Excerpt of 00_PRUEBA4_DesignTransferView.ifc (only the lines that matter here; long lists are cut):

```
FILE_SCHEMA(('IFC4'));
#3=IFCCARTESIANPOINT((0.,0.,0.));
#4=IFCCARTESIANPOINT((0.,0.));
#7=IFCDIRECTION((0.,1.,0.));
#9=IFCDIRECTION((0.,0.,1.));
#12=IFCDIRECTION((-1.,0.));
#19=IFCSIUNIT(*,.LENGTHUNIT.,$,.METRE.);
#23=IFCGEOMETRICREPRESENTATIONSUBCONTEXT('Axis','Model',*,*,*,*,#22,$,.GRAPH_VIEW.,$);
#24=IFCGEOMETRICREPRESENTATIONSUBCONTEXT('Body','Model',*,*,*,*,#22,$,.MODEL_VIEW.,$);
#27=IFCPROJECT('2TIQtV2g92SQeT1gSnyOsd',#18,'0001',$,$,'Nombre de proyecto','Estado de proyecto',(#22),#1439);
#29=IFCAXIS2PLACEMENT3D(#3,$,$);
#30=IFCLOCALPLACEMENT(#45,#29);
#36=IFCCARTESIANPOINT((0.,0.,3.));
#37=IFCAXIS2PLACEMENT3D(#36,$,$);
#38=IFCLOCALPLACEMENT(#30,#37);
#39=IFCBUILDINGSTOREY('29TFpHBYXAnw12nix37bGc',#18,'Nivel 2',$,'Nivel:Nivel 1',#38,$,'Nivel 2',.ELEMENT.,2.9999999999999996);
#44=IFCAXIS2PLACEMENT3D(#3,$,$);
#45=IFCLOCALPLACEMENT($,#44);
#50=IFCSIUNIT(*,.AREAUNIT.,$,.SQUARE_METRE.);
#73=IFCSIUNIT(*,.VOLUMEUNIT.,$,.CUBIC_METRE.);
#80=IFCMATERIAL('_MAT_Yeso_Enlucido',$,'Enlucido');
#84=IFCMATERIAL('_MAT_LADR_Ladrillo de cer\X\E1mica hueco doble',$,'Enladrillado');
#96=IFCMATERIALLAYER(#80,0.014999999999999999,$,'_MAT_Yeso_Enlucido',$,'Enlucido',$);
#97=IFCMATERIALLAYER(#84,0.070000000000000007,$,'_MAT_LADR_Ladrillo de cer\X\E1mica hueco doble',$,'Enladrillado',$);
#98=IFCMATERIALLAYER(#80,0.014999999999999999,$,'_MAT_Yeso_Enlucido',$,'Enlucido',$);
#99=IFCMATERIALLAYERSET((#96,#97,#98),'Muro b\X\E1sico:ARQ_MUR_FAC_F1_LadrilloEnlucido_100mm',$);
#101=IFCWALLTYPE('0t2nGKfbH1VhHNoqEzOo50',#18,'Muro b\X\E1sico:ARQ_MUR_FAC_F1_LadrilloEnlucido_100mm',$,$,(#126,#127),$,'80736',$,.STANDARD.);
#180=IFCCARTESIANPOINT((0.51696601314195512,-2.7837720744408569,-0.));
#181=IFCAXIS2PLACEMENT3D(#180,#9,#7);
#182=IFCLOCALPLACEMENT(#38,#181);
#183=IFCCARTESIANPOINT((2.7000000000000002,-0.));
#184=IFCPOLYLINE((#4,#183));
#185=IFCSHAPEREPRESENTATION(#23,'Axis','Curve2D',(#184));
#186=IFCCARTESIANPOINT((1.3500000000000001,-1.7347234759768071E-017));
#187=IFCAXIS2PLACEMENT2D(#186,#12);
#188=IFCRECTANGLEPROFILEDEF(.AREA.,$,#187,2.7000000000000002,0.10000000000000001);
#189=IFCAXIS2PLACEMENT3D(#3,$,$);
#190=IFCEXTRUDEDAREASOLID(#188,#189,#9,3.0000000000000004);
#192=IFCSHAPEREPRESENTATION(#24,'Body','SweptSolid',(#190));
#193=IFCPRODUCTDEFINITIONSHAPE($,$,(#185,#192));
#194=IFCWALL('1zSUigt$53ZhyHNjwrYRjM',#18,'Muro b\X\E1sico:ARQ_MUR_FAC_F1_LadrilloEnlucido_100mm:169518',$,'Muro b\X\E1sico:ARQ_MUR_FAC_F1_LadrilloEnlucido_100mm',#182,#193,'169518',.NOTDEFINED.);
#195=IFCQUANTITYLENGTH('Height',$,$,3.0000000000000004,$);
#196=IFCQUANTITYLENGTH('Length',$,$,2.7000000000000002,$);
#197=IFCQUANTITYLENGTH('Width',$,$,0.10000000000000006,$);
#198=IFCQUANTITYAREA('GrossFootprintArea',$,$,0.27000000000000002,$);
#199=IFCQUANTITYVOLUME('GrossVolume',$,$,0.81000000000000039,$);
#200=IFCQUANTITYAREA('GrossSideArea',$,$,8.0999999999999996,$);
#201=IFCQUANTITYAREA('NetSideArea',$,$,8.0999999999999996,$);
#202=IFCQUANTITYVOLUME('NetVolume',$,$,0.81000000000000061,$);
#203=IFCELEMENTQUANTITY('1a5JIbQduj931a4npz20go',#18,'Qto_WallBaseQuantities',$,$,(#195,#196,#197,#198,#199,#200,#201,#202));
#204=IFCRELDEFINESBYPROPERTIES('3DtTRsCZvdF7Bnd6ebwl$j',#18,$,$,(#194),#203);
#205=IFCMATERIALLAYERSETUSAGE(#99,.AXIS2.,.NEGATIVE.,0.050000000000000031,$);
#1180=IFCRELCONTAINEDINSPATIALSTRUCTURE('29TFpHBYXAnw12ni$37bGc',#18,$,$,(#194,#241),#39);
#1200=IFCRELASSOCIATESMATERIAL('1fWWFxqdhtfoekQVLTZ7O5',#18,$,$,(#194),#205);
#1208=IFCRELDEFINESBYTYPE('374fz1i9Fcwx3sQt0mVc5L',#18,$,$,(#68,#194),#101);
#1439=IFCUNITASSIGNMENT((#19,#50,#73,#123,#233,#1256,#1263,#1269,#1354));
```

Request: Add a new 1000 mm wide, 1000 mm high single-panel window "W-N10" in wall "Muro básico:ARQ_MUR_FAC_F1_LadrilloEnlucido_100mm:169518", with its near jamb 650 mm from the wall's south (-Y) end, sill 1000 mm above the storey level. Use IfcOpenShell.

```python
import numpy as np
import ifcopenshell
import ifcopenshell.api.feature
import ifcopenshell.api.geometry
import ifcopenshell.api.pset
import ifcopenshell.api.root
import ifcopenshell.api.spatial
import ifcopenshell.geom
import ifcopenshell.util.element
import ifcopenshell.util.placement
import ifcopenshell.util.representation
import ifcopenshell.util.shape
import ifcopenshell.util.unit

model = ifcopenshell.open("00_PRUEBA4_DesignTransferView.ifc")
unit_scale = ifcopenshell.util.unit.calculate_unit_scale(model)
area_scale = ifcopenshell.util.unit.calculate_unit_scale(model, "AREAUNIT")
volume_scale = ifcopenshell.util.unit.calculate_unit_scale(model, "VOLUMEUNIT")
settings = ifcopenshell.geom.settings()


def volume(element):
    """Net volume in cubic metres, openings subtracted."""
    shape = ifcopenshell.geom.create_shape(settings, element)
    return ifcopenshell.util.shape.get_volume(shape.geometry)


wall = model.by_guid("1zSUigt$53ZhyHNjwrYRjM")
storey = ifcopenshell.util.element.get_container(wall, ifc_class="IfcBuildingStorey")
context = ifcopenshell.util.representation.get_context(model, "Model", "Body", "MODEL_VIEW")
before = volume(wall)

width, height, from_end, sill = 1, 1, 0.65, 1  # metres

# The wall runs along its own X axis, and the end named is its -X end.
wall_shape = ifcopenshell.geom.create_shape(settings, wall)
x, y, z = ifcopenshell.util.shape.get_vertices(wall_shape.geometry).T
start = x.min() + from_end
face, thickness = float(y.min()), float(y.max() - y.min())
wall_matrix = ifcopenshell.util.placement.get_local_placement(wall.ObjectPlacement)
level = ifcopenshell.util.placement.get_local_placement(storey.ObjectPlacement)[2, 3]


def in_wall(x, y):
    """Placement at x, y metres in the wall's axes, at sill height."""
    matrix = wall_matrix.copy()
    matrix[:, 3] = wall_matrix @ np.array([x / unit_scale, y / unit_scale, 0.0, 1.0])
    matrix[2, 3] = level + sill / unit_scale
    return matrix


# Opening: a box that overshoots both wall faces by 50 mm.
opening = ifcopenshell.api.root.create_entity(model, ifc_class="IfcOpeningElement", predefined_type="OPENING")
box = ifcopenshell.api.geometry.add_wall_representation(
    model, context=context, length=width, height=height, thickness=thickness + 0.1
)
ifcopenshell.api.geometry.assign_representation(model, product=opening, representation=box)
ifcopenshell.api.geometry.edit_object_placement(model, product=opening, matrix=in_wall(start, face - 0.05), is_si=False)
ifcopenshell.api.feature.add_feature(model, feature=opening, element=wall)

window = ifcopenshell.api.root.create_entity(model, ifc_class="IfcWindow", name="W-N10", predefined_type="WINDOW")
window.OverallWidth, window.OverallHeight = width / unit_scale, height / unit_scale
window.PartitioningType = "SINGLE_PANEL"
body = ifcopenshell.api.geometry.add_window_representation(
    model,
    context=context,
    overall_width=window.OverallWidth,
    overall_height=window.OverallHeight,
    partition_type="SINGLE_PANEL",
)
ifcopenshell.api.geometry.assign_representation(model, product=window, representation=body)
ifcopenshell.api.spatial.assign_container(model, products=[window], relating_structure=storey)
ifcopenshell.api.feature.add_filling(model, opening=opening, element=window)

# Centre the window in the wall's thickness.
ifcopenshell.api.geometry.edit_object_placement(model, product=window, matrix=in_wall(start, face), is_si=False)
window_shape = ifcopenshell.geom.create_shape(settings, window)
depth = ifcopenshell.util.shape.get_vertices(window_shape.geometry)[:, 1]
offset = face + thickness / 2 - (depth.min() + depth.max()) / 2
ifcopenshell.api.geometry.edit_object_placement(model, product=window, matrix=in_wall(start, offset), is_si=False)

after = volume(wall)

# Update the wall's stored quantities.
qto = model.by_id(ifcopenshell.util.element.get_pset(wall, "Qto_WallBaseQuantities", should_inherit=False)["id"])
ifcopenshell.api.pset.edit_qto(model, qto=qto, properties={
    "NetSideArea": after / thickness / area_scale,
    "NetVolume": after / volume_scale,
})

print(f"wall volume {before:.3f} -> {after:.3f} m3")

model.write("00_PRUEBA4_DesignTransferView_v2.ifc")
```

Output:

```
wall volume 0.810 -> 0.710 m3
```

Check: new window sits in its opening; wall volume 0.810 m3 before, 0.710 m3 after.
